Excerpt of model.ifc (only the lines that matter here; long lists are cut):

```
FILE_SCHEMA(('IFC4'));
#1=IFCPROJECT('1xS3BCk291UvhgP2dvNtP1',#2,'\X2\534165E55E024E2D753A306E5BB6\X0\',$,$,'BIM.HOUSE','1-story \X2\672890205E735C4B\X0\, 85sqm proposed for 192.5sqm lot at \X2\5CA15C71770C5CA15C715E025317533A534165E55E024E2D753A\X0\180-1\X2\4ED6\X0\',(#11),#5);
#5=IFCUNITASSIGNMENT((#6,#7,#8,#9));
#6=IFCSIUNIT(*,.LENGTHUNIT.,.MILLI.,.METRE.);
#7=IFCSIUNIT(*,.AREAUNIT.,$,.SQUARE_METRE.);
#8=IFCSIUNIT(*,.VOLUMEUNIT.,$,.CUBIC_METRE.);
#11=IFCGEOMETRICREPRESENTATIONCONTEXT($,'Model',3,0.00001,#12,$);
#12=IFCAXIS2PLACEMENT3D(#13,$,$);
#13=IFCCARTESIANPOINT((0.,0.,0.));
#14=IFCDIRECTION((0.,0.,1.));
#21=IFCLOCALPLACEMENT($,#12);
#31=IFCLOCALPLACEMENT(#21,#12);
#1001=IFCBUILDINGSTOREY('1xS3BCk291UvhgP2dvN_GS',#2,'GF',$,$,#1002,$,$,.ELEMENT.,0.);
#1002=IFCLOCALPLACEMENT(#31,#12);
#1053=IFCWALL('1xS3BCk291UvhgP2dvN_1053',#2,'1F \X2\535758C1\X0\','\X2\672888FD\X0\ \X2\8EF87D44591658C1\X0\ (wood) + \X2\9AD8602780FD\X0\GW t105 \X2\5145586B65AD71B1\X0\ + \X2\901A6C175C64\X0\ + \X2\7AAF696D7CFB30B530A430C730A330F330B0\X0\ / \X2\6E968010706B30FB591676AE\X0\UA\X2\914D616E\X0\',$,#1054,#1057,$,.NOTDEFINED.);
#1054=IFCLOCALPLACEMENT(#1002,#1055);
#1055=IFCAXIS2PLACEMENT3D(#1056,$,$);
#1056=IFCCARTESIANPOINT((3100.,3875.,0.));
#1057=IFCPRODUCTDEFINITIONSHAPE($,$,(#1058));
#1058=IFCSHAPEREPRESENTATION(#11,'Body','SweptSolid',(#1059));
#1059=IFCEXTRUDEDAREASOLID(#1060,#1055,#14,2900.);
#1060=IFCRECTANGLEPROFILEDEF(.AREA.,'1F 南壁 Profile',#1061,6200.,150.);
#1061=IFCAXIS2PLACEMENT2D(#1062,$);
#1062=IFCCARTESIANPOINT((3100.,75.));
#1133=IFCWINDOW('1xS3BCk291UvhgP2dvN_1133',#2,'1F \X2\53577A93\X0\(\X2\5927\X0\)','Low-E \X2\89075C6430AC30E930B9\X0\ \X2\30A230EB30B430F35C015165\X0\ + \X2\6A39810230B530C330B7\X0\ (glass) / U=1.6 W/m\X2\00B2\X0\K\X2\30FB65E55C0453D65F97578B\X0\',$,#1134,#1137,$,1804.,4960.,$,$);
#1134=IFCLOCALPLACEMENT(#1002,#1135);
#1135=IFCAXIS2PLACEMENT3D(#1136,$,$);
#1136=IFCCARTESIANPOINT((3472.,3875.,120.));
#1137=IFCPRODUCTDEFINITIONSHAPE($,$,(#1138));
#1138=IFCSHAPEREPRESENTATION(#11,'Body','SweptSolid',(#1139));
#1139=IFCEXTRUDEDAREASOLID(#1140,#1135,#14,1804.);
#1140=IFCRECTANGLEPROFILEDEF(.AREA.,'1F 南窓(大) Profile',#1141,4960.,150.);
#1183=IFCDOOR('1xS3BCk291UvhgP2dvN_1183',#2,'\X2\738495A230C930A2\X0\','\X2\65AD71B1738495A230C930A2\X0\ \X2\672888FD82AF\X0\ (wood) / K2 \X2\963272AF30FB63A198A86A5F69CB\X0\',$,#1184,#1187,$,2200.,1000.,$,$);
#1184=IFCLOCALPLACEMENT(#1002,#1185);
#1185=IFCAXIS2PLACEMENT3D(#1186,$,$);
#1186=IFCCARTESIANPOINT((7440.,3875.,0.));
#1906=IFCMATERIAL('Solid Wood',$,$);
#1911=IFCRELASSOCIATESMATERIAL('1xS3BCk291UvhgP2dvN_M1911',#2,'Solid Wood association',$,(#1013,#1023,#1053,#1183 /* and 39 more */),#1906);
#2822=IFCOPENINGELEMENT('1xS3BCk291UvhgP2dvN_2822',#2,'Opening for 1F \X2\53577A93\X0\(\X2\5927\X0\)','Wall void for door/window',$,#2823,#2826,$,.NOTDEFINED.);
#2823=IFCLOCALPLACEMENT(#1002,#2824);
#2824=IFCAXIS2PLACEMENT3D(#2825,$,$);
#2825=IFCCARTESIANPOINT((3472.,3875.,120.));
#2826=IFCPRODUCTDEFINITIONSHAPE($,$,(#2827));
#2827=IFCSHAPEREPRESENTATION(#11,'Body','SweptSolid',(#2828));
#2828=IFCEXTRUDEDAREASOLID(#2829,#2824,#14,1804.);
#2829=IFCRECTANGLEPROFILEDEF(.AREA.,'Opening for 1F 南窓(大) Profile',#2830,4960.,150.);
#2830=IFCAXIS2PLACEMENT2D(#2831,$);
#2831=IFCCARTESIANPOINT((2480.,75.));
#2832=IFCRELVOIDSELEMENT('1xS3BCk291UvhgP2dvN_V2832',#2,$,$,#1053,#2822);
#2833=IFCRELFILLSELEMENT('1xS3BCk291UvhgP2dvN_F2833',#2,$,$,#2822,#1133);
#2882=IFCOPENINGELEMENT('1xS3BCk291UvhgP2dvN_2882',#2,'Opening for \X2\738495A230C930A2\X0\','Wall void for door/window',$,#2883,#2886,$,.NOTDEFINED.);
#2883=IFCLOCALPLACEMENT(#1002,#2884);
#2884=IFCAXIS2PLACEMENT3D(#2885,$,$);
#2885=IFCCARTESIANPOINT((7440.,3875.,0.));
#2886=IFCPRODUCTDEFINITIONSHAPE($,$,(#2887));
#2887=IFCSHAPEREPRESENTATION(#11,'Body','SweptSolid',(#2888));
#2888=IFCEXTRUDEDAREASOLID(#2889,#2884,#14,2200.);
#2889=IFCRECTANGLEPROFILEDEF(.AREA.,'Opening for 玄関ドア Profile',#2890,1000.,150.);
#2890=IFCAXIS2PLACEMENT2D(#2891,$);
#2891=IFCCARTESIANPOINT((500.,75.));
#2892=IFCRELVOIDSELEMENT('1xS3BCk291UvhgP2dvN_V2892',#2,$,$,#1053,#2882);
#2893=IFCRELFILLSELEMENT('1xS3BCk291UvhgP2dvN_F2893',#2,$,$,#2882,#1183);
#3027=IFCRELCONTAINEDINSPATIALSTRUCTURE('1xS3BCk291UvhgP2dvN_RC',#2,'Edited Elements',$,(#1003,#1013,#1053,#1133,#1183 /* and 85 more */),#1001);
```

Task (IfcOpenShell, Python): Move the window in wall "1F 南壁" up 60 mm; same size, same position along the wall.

```python
import numpy as np
import ifcopenshell
import ifcopenshell.api.geometry
import ifcopenshell.util.placement
import ifcopenshell.util.unit

model = ifcopenshell.open("model.ifc")
unit_scale = ifcopenshell.util.unit.calculate_unit_scale(model)

window = model.by_guid("1xS3BCk291UvhgP2dvN_1133")
opening = window.FillsVoids[0].RelatingOpeningElement
dz = 0.06 / unit_scale

shift = np.array([0.0, 0.0, dz])
# The window is not placed relative to its opening, so move both.
for product in (opening, window):
    matrix = ifcopenshell.util.placement.get_local_placement(product.ObjectPlacement)
    matrix[:3, 3] += shift
    ifcopenshell.api.geometry.edit_object_placement(model, product=product, matrix=matrix, is_si=False)

print(f"moved by {dz * unit_scale:+.3f} m")

model.write("model_v2.ifc")
```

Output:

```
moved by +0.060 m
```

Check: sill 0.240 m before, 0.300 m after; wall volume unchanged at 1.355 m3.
